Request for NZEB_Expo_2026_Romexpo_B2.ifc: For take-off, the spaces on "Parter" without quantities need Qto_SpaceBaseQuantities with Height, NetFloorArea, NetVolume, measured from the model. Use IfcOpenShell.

First a look at what the model holds.

```python
import ifcopenshell
import ifcopenshell.util.element
import ifcopenshell.util.unit

model = ifcopenshell.open("NZEB_Expo_2026_Romexpo_B2.ifc")
print(model.schema)
for unit_type in ("LENGTHUNIT", "AREAUNIT", "VOLUMEUNIT"):
    print(unit_type, ifcopenshell.util.unit.calculate_unit_scale(model, unit_type))
storey = next(s for s in model.by_type("IfcBuildingStorey") if s.Name == "Parter")
spaces = [e for e in ifcopenshell.util.element.get_decomposition(storey) if e.is_a("IfcSpace")]
for e in sorted(spaces, key=lambda e: e.id()):
    print(e.id(), e.is_a(), e.Name, list(ifcopenshell.util.element.get_psets(e, qtos_only=True)), sep=" | ")
```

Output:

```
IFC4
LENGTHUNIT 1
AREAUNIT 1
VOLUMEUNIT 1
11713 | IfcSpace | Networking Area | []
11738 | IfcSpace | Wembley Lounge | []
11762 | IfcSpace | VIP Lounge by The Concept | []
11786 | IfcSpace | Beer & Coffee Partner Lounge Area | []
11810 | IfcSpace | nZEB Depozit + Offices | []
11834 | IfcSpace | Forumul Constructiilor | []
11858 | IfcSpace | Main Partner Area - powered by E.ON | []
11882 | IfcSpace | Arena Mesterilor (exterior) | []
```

```python
import ifcopenshell
import ifcopenshell.api.pset
import ifcopenshell.geom
import ifcopenshell.util.element
import ifcopenshell.util.shape
import ifcopenshell.util.unit

model = ifcopenshell.open("NZEB_Expo_2026_Romexpo_B2.ifc")
unit_scale = ifcopenshell.util.unit.calculate_unit_scale(model)
area_scale = ifcopenshell.util.unit.calculate_unit_scale(model, "AREAUNIT")
volume_scale = ifcopenshell.util.unit.calculate_unit_scale(model, "VOLUMEUNIT")
settings = ifcopenshell.geom.settings()

storey = next(s for s in model.by_type("IfcBuildingStorey") if s.Name == "Parter")
spaces = [e for e in ifcopenshell.util.element.get_decomposition(storey) if e.is_a("IfcSpace")]

for e in sorted(spaces, key=lambda e: e.id()):
    if ifcopenshell.util.element.get_psets(e, qtos_only=True, should_inherit=False):
        continue
    # Geometry comes back in metres, in the element's own axes.
    shape = ifcopenshell.geom.create_shape(settings, e)
    values = {
        "Height": ifcopenshell.util.shape.get_z(shape.geometry) / unit_scale,
        "NetFloorArea": ifcopenshell.util.shape.get_footprint_area(shape.geometry) / area_scale,
        "NetVolume": ifcopenshell.util.shape.get_volume(shape.geometry) / volume_scale,
    }
    qto = ifcopenshell.api.pset.add_qto(model, product=e, name="Qto_SpaceBaseQuantities")
    ifcopenshell.api.pset.edit_qto(model, qto=qto, properties=values)
    print(e.id(), {k: round(v, 3) for k, v in values.items()})

model.write("NZEB_Expo_2026_Romexpo_B2_v2.ifc")
```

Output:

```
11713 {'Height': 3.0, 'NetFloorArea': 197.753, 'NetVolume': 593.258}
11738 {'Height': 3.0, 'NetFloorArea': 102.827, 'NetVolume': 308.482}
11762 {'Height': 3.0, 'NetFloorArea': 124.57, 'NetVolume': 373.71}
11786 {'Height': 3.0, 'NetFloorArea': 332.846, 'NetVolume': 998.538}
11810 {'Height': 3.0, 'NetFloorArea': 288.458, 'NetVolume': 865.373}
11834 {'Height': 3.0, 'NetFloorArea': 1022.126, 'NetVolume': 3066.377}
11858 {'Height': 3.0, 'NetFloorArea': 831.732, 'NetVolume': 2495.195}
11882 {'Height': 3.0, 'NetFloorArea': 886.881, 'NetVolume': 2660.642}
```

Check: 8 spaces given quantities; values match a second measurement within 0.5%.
